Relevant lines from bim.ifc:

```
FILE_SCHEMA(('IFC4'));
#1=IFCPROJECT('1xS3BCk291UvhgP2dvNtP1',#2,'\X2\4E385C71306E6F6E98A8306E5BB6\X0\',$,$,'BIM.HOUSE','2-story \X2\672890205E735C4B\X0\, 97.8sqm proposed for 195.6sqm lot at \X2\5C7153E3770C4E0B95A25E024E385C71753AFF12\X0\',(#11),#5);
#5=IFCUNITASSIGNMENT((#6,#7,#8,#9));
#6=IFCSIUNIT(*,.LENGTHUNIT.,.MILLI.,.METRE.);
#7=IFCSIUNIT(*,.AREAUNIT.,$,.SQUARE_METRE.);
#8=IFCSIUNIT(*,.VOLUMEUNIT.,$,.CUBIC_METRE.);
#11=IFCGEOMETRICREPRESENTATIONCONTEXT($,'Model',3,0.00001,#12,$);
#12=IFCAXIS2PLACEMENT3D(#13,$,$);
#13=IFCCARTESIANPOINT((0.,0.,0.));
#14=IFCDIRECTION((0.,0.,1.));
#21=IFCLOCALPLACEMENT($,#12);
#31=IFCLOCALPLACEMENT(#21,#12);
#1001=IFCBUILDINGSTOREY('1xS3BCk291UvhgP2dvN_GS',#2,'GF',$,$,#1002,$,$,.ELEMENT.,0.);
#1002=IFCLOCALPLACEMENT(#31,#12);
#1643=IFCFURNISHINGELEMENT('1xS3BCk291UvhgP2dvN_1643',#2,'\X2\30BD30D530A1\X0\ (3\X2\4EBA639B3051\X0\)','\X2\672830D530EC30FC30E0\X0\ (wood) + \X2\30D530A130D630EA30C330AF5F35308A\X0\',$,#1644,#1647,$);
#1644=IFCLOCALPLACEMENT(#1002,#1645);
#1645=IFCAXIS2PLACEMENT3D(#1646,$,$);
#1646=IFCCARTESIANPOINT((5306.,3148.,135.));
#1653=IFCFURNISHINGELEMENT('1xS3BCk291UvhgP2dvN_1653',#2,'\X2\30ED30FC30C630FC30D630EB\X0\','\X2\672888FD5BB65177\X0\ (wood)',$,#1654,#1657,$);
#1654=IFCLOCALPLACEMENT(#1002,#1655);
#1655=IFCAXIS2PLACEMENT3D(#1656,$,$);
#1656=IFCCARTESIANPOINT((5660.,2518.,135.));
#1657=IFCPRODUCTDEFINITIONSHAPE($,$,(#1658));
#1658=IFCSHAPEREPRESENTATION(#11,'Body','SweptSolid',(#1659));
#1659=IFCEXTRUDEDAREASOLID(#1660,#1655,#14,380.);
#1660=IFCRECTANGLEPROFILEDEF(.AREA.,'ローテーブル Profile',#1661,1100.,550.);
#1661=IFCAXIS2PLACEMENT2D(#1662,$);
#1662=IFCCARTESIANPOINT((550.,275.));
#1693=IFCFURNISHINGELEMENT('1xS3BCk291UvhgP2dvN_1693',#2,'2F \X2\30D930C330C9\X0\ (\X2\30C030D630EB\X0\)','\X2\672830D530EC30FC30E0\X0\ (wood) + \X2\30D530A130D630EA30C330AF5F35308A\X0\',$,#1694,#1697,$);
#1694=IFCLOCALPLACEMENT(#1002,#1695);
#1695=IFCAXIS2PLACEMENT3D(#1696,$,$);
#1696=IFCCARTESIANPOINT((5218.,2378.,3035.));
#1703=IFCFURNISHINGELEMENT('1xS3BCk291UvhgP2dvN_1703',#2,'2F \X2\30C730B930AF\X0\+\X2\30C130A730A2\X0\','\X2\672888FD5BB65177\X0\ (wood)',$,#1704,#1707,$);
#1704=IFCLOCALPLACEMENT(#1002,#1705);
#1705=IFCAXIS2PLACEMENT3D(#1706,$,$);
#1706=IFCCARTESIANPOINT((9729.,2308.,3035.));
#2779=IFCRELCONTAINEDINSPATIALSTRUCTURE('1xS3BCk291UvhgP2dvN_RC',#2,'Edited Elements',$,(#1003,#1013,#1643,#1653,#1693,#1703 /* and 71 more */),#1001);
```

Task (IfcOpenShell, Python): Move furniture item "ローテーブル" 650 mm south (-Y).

```python
import ifcopenshell
import ifcopenshell.api.geometry
import ifcopenshell.util.placement
import ifcopenshell.util.unit

model = ifcopenshell.open("bim.ifc")
unit_scale = ifcopenshell.util.unit.calculate_unit_scale(model)

item = model.by_guid("1xS3BCk291UvhgP2dvN_1653")
matrix = ifcopenshell.util.placement.get_local_placement(item.ObjectPlacement)
matrix[1, 3] -= 0.65 / unit_scale
ifcopenshell.api.geometry.edit_object_placement(model, product=item, matrix=matrix, is_si=False)

print(ifcopenshell.util.placement.get_local_placement(item.ObjectPlacement).round(3) + 0.0)

model.write("bim_v2.ifc")
```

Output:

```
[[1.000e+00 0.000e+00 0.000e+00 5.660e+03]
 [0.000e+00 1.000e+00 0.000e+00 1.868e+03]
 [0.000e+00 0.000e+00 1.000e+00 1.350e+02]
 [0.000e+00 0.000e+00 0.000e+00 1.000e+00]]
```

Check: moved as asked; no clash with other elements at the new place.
